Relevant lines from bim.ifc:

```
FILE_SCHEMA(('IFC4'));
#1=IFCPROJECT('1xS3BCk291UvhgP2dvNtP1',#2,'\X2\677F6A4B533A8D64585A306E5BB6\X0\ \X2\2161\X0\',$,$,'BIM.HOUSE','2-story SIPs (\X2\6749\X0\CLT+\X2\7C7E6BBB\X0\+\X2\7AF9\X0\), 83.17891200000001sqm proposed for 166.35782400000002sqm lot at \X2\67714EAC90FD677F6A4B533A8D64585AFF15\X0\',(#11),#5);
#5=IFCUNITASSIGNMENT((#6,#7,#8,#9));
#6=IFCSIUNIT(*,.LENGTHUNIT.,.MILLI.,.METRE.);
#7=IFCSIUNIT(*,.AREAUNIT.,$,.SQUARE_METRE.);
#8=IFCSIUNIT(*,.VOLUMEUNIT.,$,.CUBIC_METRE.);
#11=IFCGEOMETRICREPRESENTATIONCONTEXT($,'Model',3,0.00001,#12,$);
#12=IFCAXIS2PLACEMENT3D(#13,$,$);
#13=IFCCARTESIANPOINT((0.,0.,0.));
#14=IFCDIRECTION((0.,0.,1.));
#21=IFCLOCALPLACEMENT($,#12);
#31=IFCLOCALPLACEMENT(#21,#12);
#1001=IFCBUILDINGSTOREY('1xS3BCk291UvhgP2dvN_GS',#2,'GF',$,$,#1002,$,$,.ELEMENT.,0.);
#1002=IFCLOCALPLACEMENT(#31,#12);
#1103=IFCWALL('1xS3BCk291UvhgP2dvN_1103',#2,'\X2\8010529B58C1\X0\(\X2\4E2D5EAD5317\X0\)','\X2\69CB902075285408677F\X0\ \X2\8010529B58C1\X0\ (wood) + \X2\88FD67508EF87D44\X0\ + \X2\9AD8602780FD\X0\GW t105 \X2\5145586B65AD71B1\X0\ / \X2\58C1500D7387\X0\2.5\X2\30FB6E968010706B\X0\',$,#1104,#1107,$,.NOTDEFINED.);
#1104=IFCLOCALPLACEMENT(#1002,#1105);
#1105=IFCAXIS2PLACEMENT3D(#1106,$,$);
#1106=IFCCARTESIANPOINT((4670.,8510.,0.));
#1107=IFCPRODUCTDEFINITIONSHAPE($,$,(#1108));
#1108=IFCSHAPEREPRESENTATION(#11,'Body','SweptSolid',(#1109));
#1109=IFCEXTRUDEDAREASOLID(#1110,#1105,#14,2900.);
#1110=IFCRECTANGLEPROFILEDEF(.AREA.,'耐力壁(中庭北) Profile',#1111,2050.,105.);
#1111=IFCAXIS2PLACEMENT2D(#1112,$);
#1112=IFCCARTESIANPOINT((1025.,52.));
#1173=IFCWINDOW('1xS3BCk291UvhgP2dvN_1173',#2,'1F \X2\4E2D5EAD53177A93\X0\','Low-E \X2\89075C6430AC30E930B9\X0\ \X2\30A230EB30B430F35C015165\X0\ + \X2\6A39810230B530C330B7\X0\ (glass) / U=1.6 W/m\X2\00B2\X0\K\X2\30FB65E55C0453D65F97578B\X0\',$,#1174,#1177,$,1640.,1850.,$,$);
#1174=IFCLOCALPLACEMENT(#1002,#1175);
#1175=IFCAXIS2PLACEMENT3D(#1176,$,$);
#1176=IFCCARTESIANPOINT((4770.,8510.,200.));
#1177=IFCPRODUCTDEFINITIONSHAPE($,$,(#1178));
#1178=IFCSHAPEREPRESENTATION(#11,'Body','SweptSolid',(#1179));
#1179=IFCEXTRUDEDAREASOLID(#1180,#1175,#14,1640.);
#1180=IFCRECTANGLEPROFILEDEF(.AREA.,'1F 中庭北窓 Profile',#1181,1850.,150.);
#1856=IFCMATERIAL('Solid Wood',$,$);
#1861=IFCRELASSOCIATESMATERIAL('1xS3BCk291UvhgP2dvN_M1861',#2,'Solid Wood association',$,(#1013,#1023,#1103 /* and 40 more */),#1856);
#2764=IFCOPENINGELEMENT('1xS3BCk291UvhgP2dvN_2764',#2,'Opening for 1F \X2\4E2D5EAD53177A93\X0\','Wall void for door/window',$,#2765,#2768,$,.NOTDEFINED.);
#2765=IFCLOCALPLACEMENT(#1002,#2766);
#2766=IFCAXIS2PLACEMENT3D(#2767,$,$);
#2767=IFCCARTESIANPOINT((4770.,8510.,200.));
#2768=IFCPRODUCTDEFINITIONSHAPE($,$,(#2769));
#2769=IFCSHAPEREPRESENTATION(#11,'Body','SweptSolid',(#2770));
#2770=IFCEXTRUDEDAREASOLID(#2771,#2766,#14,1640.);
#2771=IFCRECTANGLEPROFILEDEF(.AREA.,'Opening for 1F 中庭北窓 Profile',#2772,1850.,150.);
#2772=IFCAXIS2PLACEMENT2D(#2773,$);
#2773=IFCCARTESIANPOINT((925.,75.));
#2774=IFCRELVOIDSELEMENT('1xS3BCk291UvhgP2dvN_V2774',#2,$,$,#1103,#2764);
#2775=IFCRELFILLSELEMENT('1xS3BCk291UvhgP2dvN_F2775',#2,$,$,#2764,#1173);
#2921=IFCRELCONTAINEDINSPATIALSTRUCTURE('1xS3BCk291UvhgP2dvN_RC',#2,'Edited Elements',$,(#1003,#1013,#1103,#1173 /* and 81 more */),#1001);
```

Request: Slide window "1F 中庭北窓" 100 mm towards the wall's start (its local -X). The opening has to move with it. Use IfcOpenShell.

```python
import ifcopenshell
import ifcopenshell.api.geometry
import ifcopenshell.util.placement

model = ifcopenshell.open("bim.ifc")

window = model.by_guid("1xS3BCk291UvhgP2dvN_1173")
opening = window.FillsVoids[0].RelatingOpeningElement
wall = opening.VoidsElements[0].RelatingBuildingElement

wall_matrix = ifcopenshell.util.placement.get_local_placement(wall.ObjectPlacement)
shift = wall_matrix[:3, 0] * -100.0
before = ifcopenshell.util.placement.get_local_placement(window.ObjectPlacement)[:3, 3].copy()

# The window is not placed relative to its opening, so move both.
for product in (opening, window):
    matrix = ifcopenshell.util.placement.get_local_placement(product.ObjectPlacement)
    matrix[:3, 3] += shift
    ifcopenshell.api.geometry.edit_object_placement(model, product=product, matrix=matrix, is_si=False)

after = ifcopenshell.util.placement.get_local_placement(window.ObjectPlacement)[:3, 3]
print("window moved by", (after - before).round(3) + 0.0)

model.write("bim_edited.ifc")
```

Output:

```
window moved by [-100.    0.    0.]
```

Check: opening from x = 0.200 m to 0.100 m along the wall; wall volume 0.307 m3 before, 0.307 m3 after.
